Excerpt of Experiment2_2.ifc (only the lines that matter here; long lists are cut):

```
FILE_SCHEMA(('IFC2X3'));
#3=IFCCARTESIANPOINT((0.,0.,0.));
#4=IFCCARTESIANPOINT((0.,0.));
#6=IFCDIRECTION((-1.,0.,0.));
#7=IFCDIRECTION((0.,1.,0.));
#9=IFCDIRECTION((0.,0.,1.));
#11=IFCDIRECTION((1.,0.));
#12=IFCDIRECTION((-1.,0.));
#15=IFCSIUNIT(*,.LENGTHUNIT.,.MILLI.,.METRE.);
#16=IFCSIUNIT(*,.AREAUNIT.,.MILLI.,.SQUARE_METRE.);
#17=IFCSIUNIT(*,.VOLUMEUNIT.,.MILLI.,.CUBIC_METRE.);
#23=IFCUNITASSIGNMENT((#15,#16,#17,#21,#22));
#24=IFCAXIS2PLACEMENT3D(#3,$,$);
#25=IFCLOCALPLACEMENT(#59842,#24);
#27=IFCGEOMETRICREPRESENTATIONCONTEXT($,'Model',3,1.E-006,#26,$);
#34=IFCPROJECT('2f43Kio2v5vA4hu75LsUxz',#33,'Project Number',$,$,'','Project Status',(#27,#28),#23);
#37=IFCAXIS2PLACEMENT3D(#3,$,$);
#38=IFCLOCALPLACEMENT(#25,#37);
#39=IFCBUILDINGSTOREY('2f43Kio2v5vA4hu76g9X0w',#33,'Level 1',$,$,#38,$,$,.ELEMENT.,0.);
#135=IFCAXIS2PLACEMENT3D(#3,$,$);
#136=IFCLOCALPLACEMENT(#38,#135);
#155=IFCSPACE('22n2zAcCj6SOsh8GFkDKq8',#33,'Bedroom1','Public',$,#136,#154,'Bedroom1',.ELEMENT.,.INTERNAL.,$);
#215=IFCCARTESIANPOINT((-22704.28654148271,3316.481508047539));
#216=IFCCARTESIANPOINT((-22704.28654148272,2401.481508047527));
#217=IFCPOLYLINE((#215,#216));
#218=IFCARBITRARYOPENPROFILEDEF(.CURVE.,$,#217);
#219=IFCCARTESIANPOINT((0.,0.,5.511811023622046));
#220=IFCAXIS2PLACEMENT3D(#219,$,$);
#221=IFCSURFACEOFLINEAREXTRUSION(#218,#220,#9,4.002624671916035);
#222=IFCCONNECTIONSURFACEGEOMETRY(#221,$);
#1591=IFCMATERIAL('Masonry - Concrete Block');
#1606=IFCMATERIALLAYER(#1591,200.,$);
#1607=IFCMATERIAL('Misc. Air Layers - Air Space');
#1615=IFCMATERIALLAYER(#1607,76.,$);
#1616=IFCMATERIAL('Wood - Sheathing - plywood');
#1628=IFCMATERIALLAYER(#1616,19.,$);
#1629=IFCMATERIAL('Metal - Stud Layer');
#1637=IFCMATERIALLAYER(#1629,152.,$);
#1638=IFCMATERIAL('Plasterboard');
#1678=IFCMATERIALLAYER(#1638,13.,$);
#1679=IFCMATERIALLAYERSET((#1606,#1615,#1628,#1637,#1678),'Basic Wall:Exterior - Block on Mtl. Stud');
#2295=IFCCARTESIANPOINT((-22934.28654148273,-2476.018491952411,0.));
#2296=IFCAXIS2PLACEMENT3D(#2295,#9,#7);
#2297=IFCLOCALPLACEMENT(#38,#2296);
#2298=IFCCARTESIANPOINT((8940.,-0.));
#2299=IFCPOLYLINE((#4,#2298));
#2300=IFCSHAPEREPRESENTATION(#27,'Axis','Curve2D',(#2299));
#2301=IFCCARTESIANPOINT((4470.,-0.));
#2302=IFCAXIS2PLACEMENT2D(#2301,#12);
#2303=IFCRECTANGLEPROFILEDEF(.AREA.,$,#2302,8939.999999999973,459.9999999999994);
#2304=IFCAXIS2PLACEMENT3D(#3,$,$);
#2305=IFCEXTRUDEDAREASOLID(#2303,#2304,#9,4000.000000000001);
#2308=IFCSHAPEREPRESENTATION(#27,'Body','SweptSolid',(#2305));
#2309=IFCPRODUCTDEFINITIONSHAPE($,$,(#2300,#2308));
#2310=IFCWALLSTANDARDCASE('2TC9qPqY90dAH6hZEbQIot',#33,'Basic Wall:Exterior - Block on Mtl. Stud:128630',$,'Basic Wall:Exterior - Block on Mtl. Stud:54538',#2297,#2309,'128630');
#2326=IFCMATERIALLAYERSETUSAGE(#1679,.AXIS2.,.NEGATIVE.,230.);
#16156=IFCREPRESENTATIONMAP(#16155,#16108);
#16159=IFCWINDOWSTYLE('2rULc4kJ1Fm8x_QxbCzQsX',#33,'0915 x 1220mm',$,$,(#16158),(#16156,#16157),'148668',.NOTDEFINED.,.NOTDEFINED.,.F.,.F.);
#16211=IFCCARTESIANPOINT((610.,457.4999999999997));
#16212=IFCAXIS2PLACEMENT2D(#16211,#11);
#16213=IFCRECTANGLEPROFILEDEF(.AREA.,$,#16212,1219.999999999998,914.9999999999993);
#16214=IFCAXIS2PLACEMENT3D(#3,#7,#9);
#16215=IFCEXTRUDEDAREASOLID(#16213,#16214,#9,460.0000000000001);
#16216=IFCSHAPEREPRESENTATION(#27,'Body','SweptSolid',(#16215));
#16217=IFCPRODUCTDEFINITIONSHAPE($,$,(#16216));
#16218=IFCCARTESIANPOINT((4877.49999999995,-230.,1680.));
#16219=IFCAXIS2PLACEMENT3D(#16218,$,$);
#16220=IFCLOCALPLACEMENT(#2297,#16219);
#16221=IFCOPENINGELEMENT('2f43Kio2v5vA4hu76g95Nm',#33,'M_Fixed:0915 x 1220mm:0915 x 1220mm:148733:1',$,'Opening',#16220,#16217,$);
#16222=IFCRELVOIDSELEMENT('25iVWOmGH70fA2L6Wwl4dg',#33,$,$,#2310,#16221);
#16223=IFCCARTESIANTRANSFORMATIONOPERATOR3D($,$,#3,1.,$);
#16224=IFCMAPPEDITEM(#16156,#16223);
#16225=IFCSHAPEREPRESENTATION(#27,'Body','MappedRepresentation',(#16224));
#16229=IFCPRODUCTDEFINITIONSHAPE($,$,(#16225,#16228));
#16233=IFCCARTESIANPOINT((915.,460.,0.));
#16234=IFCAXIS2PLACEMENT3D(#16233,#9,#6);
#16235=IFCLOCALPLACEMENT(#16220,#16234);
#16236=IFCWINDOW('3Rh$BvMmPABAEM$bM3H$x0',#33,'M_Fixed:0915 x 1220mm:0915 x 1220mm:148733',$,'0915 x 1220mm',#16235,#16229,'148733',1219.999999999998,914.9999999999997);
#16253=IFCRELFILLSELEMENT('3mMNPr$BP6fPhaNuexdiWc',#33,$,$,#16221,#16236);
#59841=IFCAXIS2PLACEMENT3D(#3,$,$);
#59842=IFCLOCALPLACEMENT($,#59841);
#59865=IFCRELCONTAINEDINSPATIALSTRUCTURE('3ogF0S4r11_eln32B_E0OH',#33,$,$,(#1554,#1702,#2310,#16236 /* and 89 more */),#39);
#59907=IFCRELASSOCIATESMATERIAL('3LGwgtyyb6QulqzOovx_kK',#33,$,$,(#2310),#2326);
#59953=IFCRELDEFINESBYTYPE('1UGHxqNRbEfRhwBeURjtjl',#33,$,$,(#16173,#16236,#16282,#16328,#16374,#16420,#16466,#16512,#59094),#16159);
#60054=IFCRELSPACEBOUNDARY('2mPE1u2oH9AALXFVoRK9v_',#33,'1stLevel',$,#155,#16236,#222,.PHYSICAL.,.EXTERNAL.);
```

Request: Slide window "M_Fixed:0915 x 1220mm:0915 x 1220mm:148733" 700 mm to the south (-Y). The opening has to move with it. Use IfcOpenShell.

```python
import numpy as np
import ifcopenshell
import ifcopenshell.api.geometry
import ifcopenshell.util.placement
import ifcopenshell.util.unit

model = ifcopenshell.open("Experiment2_2.ifc")
unit_scale = ifcopenshell.util.unit.calculate_unit_scale(model)

window = model.by_id(16236)
opening = window.FillsVoids[0].RelatingOpeningElement
wall = opening.VoidsElements[0].RelatingBuildingElement

wall_matrix = ifcopenshell.util.placement.get_local_placement(wall.ObjectPlacement)
shift = wall_matrix[:3, 0] * -0.7 / unit_scale
before = ifcopenshell.util.placement.get_local_placement(window.ObjectPlacement)[:3, 3].copy()

# The window is placed relative to its opening, so it follows when the opening moves.
matrix = ifcopenshell.util.placement.get_local_placement(opening.ObjectPlacement)
matrix[:3, 3] += shift
ifcopenshell.api.geometry.edit_object_placement(
    model, product=opening, matrix=matrix, is_si=False, should_transform_children=True
)

# Space boundary surfaces are stored in each space's coordinates; move them too.
for rel in window.ProvidesBoundaries:
    if not rel.ConnectionGeometry:
        continue
    surface = rel.ConnectionGeometry.SurfaceOnRelatingElement
    space_matrix = ifcopenshell.util.placement.get_local_placement(rel.RelatingSpace.ObjectPlacement)
    point = np.array(surface.Position.Location.Coordinates) + space_matrix[:3, :3].T @ shift
    surface.Position = model.createIfcAxis2Placement3D(
        model.createIfcCartesianPoint(point.tolist()), surface.Position.Axis, surface.Position.RefDirection
    )

after = ifcopenshell.util.placement.get_local_placement(window.ObjectPlacement)[:3, 3]
print("window moved by", (after - before).round(3) + 0.0)

model.write("Experiment2_2_edited.ifc")
```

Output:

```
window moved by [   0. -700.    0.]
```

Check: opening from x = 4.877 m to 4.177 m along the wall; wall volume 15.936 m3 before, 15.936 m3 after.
